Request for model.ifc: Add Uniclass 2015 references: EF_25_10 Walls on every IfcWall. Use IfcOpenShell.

First a look at what the model holds.

```python
import ifcopenshell

model = ifcopenshell.open("model.ifc")
print(model.schema)
print("classifications:", [c.Name for c in model.by_type("IfcClassification")])
for ifc_class in ("IfcDoor", "IfcRoof", "IfcStair", "IfcWall", "IfcWindow"):
    print(ifc_class, len(model.by_type(ifc_class)))
```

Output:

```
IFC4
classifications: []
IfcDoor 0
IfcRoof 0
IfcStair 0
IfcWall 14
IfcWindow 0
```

```python
import ifcopenshell
import ifcopenshell.api.classification

model = ifcopenshell.open("model.ifc")

system = ifcopenshell.api.classification.add_classification(model, classification="Uniclass 2015")

codes = {
    "IfcWall": ("EF_25_10", "Walls"),
}
for ifc_class, (code, name) in codes.items():
    products = model.by_type(ifc_class)
    ifcopenshell.api.classification.add_reference(
        model, products=products, classification=system, identification=code, name=name
    )
    print(code, len(products))

model.write("model_v2.ifc")
```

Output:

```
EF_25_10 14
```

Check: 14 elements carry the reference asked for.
